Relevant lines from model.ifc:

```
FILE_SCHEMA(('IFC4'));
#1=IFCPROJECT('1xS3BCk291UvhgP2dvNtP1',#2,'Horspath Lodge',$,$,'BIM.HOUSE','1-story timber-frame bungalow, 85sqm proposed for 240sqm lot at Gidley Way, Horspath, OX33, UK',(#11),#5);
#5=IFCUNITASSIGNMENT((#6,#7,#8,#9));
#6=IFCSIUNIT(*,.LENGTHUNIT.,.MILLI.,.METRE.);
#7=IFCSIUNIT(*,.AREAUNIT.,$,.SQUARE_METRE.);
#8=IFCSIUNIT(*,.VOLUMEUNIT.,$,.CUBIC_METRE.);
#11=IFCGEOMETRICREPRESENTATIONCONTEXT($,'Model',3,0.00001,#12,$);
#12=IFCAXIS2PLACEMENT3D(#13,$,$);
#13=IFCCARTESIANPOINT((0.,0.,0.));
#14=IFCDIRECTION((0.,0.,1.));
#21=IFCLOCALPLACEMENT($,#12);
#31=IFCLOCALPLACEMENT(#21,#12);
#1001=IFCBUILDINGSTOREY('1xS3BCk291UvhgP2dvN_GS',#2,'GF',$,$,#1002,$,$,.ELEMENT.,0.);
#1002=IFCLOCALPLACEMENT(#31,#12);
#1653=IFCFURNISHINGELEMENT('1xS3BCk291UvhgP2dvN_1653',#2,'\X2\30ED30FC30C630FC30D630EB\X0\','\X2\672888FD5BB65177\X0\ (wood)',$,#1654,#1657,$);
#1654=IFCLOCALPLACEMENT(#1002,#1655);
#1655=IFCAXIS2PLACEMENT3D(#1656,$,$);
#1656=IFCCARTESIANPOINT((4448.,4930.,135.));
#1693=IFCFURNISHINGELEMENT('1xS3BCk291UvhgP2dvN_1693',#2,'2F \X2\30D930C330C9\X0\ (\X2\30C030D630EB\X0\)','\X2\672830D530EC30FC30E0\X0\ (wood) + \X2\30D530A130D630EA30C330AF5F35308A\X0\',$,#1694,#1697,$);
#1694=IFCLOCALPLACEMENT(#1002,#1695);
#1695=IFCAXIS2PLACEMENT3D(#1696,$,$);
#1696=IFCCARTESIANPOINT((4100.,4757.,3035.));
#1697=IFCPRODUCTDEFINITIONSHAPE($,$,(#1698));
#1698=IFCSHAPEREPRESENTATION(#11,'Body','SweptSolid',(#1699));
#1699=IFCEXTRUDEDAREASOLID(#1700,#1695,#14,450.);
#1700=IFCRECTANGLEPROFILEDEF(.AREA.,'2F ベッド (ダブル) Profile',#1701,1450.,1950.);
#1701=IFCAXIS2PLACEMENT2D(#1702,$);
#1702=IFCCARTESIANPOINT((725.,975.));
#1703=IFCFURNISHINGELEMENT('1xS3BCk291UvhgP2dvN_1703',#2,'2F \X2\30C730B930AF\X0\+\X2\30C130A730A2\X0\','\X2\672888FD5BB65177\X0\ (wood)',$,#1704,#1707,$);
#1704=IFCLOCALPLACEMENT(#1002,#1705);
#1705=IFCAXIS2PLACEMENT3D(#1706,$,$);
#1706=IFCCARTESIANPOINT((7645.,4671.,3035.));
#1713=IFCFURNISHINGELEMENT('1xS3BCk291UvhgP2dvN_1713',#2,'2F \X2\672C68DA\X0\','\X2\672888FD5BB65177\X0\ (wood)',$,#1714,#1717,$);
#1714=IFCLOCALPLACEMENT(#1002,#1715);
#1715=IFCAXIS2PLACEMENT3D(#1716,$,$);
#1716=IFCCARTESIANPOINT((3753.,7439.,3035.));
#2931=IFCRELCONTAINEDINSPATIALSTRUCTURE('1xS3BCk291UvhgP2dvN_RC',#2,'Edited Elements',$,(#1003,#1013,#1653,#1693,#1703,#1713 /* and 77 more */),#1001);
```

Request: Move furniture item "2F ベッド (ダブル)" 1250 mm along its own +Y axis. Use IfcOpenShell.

```python
import ifcopenshell
import ifcopenshell.api.geometry
import ifcopenshell.util.placement
import ifcopenshell.util.unit

model = ifcopenshell.open("model.ifc")
unit_scale = ifcopenshell.util.unit.calculate_unit_scale(model)

item = model.by_guid("1xS3BCk291UvhgP2dvN_1693")
matrix = ifcopenshell.util.placement.get_local_placement(item.ObjectPlacement)
matrix[:3, 3] += matrix[:3, 1] * 1.25 / unit_scale
ifcopenshell.api.geometry.edit_object_placement(model, product=item, matrix=matrix, is_si=False)

print(ifcopenshell.util.placement.get_local_placement(item.ObjectPlacement).round(3) + 0.0)

model.write("model_updated.ifc")
```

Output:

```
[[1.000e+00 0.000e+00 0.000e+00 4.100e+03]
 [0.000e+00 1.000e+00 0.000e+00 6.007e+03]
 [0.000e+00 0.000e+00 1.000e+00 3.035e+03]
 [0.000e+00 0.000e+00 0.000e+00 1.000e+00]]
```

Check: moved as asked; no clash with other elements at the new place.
